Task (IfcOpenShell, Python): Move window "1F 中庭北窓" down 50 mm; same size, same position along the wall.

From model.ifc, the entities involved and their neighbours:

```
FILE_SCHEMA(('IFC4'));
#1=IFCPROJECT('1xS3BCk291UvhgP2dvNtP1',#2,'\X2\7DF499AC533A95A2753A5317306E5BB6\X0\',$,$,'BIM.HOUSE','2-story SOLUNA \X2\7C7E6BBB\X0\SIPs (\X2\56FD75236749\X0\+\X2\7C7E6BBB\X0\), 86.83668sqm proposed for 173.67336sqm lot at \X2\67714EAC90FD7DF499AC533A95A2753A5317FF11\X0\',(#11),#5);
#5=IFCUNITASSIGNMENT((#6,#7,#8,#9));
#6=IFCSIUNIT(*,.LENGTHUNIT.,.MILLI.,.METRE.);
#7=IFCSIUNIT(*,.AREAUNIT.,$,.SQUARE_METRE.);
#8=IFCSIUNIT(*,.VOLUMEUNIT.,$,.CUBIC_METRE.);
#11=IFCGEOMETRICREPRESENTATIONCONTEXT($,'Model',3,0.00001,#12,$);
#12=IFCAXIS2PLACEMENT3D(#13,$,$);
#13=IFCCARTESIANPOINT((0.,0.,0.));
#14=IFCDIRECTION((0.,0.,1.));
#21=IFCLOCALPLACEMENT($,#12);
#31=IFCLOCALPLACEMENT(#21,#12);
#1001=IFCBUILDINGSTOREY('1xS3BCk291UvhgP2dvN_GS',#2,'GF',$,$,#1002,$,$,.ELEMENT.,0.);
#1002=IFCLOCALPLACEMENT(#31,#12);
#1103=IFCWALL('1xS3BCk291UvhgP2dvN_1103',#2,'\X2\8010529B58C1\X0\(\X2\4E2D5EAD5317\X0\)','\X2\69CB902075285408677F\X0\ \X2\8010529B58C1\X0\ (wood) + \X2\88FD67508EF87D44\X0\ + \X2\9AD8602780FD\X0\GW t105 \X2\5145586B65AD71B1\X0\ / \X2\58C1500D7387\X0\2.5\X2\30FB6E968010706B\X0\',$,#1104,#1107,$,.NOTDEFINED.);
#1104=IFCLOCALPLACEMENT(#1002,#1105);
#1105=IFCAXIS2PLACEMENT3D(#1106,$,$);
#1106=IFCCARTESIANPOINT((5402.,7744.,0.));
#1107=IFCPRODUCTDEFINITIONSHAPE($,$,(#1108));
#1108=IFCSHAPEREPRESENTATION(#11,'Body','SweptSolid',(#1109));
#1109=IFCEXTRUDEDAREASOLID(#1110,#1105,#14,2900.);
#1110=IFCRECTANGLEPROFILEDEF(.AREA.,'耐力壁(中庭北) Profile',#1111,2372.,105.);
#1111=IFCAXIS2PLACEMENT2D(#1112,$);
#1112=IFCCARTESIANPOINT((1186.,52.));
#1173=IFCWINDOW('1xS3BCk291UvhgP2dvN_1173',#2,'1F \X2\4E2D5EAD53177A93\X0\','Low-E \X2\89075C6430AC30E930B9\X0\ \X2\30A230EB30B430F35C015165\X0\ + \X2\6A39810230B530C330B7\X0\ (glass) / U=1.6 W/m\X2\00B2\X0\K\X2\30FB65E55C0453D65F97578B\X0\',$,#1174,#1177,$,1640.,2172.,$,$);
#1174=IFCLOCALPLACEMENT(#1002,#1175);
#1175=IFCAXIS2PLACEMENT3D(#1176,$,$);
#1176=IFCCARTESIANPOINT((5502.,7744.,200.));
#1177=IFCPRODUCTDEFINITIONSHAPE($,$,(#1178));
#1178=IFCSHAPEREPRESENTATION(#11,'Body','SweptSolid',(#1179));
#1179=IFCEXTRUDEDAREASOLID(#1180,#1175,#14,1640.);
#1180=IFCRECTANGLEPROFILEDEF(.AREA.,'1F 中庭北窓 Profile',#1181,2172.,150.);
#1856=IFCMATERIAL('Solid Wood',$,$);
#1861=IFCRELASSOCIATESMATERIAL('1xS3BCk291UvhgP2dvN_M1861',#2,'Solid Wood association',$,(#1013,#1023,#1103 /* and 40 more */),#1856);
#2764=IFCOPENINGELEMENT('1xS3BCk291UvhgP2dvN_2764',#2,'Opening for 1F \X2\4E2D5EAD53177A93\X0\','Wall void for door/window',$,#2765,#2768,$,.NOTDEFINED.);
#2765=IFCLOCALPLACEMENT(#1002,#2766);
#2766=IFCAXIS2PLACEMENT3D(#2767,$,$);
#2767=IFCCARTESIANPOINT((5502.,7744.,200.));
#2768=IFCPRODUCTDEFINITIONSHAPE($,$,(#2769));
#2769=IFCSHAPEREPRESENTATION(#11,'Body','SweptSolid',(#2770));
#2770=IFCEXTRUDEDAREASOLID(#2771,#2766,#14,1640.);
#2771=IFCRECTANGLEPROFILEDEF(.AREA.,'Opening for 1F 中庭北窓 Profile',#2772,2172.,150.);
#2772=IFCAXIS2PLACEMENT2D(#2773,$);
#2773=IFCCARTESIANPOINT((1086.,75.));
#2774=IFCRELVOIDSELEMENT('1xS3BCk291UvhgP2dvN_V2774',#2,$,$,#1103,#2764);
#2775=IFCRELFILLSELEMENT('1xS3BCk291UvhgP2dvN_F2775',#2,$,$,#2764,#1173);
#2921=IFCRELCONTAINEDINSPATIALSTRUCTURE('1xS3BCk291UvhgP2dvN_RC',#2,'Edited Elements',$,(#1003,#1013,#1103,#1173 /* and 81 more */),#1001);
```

```python
import numpy as np
import ifcopenshell
import ifcopenshell.api.geometry
import ifcopenshell.util.placement
import ifcopenshell.util.unit

model = ifcopenshell.open("model.ifc")
unit_scale = ifcopenshell.util.unit.calculate_unit_scale(model)

window = model.by_guid("1xS3BCk291UvhgP2dvN_1173")
opening = window.FillsVoids[0].RelatingOpeningElement
dz = -0.05 / unit_scale

shift = np.array([0.0, 0.0, dz])
# The window is not placed relative to its opening, so move both.
for product in (opening, window):
    matrix = ifcopenshell.util.placement.get_local_placement(product.ObjectPlacement)
    matrix[:3, 3] += shift
    ifcopenshell.api.geometry.edit_object_placement(model, product=product, matrix=matrix, is_si=False)

print(f"moved by {dz * unit_scale:+.3f} m")

model.write("model_edited.ifc")
```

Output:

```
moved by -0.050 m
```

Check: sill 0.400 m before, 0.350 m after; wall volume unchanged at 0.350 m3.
